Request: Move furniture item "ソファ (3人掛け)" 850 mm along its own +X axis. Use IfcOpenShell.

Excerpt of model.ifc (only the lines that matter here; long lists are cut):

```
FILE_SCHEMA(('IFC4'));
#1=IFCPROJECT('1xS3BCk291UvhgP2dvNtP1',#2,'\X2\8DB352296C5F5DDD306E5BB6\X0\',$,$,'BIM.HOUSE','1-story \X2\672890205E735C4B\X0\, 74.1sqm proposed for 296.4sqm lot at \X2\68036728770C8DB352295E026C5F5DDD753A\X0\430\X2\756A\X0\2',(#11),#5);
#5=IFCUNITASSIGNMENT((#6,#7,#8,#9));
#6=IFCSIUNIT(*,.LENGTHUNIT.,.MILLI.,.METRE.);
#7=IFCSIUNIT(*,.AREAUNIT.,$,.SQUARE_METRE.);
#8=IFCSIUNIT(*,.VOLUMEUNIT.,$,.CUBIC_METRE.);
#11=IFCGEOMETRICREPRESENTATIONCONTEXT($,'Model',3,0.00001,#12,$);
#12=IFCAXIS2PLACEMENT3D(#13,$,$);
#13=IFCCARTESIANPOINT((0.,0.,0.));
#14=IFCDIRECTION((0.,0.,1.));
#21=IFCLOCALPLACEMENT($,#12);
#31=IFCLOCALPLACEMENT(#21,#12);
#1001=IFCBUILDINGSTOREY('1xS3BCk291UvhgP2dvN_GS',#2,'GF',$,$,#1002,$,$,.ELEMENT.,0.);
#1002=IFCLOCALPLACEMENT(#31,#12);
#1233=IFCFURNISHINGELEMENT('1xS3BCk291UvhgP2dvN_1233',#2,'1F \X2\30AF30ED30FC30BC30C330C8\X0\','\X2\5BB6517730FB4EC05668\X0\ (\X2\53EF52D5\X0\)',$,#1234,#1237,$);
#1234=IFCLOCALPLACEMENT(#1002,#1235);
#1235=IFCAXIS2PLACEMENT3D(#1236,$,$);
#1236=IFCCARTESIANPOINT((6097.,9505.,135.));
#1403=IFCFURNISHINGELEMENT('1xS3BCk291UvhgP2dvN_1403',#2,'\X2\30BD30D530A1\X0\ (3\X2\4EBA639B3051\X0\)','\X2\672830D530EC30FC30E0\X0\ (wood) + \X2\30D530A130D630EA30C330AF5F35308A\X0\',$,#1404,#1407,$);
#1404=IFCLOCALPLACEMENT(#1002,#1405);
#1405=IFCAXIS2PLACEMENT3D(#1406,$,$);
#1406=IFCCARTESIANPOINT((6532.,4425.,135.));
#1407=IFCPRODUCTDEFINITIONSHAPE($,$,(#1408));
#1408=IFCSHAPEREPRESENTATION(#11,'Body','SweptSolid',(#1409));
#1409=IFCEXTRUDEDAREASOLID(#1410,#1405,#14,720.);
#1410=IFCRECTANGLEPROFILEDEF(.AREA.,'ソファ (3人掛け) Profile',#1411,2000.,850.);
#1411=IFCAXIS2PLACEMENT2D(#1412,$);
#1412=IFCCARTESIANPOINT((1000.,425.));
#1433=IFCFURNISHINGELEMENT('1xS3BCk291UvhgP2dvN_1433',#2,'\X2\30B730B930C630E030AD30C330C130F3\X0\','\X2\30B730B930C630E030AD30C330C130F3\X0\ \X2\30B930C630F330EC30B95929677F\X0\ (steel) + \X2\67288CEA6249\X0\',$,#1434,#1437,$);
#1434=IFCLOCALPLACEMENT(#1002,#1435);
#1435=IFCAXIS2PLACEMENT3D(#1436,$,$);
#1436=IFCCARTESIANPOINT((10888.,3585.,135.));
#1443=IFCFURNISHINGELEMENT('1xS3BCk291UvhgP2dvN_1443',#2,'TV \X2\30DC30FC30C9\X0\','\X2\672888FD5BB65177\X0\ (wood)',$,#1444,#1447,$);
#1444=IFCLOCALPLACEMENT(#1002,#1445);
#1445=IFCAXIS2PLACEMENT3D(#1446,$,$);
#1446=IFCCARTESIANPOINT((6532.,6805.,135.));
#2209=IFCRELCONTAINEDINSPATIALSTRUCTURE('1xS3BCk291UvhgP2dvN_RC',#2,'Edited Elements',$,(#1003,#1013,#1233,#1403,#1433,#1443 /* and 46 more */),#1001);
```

```python
import ifcopenshell
import ifcopenshell.api.geometry
import ifcopenshell.util.placement

model = ifcopenshell.open("model.ifc")

item = model.by_guid("1xS3BCk291UvhgP2dvN_1403")
matrix = ifcopenshell.util.placement.get_local_placement(item.ObjectPlacement)
matrix[:3, 3] += matrix[:3, 0] * 850.0
ifcopenshell.api.geometry.edit_object_placement(model, product=item, matrix=matrix, is_si=False)

print(ifcopenshell.util.placement.get_local_placement(item.ObjectPlacement).round(3) + 0.0)

model.write("model_v2.ifc")
```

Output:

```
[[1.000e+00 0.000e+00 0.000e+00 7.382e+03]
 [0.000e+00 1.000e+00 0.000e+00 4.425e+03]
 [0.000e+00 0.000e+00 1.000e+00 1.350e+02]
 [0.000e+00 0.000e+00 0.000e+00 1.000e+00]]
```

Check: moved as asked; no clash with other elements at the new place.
